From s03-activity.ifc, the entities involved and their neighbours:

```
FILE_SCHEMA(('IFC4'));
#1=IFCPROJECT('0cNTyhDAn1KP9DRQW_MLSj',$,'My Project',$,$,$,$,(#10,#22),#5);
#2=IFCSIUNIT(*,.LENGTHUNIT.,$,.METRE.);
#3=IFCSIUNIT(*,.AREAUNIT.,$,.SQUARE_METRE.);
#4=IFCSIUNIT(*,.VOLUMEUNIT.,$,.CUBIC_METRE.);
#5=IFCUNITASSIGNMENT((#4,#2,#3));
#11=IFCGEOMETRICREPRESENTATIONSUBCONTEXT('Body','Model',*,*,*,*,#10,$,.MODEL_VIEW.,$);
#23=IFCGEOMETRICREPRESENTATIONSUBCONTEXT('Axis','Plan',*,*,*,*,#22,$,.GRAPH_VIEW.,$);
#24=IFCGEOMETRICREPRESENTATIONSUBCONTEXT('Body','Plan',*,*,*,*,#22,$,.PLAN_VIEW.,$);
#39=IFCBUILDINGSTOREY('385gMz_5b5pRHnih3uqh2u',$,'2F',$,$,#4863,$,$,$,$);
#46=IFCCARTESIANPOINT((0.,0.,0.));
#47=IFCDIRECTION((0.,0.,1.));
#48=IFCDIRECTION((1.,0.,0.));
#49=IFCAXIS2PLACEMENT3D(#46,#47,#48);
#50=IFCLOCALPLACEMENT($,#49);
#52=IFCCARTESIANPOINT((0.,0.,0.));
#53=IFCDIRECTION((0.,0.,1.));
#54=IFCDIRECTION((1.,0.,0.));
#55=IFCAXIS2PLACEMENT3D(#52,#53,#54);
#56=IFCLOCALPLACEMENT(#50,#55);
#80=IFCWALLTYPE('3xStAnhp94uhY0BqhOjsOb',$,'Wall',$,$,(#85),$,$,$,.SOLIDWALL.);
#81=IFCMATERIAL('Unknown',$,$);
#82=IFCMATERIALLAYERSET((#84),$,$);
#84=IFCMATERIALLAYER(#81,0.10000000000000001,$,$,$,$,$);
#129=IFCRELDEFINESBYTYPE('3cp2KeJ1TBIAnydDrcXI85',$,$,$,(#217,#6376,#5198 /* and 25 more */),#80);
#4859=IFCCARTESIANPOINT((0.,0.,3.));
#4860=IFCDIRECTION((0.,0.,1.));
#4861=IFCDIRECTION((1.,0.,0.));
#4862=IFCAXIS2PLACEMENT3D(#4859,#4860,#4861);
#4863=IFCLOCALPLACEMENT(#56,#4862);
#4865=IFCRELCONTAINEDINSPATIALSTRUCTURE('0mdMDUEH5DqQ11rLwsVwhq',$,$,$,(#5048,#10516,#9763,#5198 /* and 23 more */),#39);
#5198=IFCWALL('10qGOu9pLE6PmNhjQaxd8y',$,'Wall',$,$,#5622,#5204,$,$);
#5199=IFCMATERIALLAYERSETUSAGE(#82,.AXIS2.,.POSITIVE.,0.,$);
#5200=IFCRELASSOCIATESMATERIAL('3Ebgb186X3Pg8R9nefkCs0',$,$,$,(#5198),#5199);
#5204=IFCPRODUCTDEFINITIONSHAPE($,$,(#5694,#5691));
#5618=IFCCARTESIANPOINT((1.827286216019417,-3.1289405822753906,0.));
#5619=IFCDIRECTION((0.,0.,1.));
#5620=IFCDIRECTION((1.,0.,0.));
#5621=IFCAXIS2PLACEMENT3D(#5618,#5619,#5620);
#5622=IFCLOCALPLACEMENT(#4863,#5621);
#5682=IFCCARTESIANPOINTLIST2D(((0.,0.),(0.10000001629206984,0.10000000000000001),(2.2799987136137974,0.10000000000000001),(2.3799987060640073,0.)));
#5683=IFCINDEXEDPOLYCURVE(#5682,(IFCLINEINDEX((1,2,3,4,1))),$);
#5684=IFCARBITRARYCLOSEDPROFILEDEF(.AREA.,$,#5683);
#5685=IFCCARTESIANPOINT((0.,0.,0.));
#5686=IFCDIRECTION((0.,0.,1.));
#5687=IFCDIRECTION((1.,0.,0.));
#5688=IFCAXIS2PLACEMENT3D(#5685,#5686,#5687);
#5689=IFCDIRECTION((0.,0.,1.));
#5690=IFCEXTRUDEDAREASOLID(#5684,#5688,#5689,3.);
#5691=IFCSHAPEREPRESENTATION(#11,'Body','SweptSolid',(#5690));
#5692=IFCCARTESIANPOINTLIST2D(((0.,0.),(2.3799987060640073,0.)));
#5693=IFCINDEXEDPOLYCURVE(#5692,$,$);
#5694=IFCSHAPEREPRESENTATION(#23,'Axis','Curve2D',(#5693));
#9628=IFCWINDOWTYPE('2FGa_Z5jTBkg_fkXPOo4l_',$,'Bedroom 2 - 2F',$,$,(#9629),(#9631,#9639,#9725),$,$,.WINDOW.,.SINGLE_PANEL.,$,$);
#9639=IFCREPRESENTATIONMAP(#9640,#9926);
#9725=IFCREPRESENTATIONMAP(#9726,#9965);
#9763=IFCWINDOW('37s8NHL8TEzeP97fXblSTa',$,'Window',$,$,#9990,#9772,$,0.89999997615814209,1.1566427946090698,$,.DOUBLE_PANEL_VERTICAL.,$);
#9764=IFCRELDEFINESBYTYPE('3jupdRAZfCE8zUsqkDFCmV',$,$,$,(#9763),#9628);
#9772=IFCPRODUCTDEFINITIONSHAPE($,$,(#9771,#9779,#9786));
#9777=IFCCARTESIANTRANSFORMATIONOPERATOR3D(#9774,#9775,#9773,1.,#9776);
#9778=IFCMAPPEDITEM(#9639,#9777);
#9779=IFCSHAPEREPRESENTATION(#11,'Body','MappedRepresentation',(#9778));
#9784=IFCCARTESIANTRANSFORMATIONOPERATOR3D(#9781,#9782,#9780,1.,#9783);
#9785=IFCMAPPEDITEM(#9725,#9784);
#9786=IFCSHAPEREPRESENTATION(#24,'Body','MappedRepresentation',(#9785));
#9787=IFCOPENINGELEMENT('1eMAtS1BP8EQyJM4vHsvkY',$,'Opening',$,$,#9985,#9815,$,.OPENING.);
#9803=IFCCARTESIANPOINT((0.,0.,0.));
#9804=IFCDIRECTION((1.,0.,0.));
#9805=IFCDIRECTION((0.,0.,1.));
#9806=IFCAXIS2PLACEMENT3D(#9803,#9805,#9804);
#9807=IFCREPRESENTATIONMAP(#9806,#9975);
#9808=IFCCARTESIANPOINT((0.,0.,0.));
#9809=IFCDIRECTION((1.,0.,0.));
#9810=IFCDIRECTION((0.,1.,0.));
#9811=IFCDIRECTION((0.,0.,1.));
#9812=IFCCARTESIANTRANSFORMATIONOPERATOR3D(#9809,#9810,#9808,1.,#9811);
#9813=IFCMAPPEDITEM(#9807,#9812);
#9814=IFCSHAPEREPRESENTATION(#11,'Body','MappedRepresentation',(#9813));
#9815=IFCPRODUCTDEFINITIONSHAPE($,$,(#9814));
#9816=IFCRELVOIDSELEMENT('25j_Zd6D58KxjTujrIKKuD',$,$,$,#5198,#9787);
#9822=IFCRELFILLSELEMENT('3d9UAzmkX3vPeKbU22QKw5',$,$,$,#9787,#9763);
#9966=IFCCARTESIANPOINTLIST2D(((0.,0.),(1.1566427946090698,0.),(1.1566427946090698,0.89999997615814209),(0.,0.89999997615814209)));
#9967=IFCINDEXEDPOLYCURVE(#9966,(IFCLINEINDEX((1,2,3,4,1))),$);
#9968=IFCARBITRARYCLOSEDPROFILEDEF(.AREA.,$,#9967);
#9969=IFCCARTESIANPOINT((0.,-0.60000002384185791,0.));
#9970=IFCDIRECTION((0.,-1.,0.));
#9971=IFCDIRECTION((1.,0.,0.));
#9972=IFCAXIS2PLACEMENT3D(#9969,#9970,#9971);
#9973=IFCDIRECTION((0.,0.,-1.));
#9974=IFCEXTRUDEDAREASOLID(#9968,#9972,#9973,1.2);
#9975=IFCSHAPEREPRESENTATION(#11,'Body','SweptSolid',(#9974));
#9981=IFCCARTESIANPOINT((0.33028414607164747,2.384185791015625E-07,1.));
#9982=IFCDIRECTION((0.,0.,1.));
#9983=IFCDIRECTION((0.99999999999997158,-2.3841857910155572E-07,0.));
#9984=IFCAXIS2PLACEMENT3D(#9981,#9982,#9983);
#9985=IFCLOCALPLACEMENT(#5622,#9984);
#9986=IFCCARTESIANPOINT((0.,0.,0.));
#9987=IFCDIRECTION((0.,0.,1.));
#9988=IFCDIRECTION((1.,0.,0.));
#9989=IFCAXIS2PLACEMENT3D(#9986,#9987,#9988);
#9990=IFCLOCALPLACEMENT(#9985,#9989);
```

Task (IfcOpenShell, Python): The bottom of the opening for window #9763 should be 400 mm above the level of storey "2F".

```python
import numpy as np
import ifcopenshell
import ifcopenshell.api.geometry
import ifcopenshell.geom
import ifcopenshell.util.element
import ifcopenshell.util.placement
import ifcopenshell.util.shape
import ifcopenshell.util.unit

model = ifcopenshell.open("s03-activity.ifc")
unit_scale = ifcopenshell.util.unit.calculate_unit_scale(model)

window = model.by_guid("37s8NHL8TEzeP97fXblSTa")
opening = window.FillsVoids[0].RelatingOpeningElement
storey = ifcopenshell.util.element.get_container(window, ifc_class="IfcBuildingStorey")
level = ifcopenshell.util.placement.get_local_placement(storey.ObjectPlacement)[2, 3]

# The opening's origin need not be at the sill, so measure its lowest point.
shape = ifcopenshell.geom.create_shape(ifcopenshell.geom.settings(), opening)
bottom = ifcopenshell.util.shape.get_shape_bottom_elevation(shape, shape.geometry) / unit_scale
dz = level + 0.4 / unit_scale - bottom

shift = np.array([0.0, 0.0, dz])
# The window is placed relative to its opening, so it follows when the opening moves.
matrix = ifcopenshell.util.placement.get_local_placement(opening.ObjectPlacement)
matrix[:3, 3] += shift
ifcopenshell.api.geometry.edit_object_placement(
    model, product=opening, matrix=matrix, is_si=False, should_transform_children=True
)

print(f"moved by {dz * unit_scale:+.3f} m")

model.write("s03-activity_edited.ifc")
```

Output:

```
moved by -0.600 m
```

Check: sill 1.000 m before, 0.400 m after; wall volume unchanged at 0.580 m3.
